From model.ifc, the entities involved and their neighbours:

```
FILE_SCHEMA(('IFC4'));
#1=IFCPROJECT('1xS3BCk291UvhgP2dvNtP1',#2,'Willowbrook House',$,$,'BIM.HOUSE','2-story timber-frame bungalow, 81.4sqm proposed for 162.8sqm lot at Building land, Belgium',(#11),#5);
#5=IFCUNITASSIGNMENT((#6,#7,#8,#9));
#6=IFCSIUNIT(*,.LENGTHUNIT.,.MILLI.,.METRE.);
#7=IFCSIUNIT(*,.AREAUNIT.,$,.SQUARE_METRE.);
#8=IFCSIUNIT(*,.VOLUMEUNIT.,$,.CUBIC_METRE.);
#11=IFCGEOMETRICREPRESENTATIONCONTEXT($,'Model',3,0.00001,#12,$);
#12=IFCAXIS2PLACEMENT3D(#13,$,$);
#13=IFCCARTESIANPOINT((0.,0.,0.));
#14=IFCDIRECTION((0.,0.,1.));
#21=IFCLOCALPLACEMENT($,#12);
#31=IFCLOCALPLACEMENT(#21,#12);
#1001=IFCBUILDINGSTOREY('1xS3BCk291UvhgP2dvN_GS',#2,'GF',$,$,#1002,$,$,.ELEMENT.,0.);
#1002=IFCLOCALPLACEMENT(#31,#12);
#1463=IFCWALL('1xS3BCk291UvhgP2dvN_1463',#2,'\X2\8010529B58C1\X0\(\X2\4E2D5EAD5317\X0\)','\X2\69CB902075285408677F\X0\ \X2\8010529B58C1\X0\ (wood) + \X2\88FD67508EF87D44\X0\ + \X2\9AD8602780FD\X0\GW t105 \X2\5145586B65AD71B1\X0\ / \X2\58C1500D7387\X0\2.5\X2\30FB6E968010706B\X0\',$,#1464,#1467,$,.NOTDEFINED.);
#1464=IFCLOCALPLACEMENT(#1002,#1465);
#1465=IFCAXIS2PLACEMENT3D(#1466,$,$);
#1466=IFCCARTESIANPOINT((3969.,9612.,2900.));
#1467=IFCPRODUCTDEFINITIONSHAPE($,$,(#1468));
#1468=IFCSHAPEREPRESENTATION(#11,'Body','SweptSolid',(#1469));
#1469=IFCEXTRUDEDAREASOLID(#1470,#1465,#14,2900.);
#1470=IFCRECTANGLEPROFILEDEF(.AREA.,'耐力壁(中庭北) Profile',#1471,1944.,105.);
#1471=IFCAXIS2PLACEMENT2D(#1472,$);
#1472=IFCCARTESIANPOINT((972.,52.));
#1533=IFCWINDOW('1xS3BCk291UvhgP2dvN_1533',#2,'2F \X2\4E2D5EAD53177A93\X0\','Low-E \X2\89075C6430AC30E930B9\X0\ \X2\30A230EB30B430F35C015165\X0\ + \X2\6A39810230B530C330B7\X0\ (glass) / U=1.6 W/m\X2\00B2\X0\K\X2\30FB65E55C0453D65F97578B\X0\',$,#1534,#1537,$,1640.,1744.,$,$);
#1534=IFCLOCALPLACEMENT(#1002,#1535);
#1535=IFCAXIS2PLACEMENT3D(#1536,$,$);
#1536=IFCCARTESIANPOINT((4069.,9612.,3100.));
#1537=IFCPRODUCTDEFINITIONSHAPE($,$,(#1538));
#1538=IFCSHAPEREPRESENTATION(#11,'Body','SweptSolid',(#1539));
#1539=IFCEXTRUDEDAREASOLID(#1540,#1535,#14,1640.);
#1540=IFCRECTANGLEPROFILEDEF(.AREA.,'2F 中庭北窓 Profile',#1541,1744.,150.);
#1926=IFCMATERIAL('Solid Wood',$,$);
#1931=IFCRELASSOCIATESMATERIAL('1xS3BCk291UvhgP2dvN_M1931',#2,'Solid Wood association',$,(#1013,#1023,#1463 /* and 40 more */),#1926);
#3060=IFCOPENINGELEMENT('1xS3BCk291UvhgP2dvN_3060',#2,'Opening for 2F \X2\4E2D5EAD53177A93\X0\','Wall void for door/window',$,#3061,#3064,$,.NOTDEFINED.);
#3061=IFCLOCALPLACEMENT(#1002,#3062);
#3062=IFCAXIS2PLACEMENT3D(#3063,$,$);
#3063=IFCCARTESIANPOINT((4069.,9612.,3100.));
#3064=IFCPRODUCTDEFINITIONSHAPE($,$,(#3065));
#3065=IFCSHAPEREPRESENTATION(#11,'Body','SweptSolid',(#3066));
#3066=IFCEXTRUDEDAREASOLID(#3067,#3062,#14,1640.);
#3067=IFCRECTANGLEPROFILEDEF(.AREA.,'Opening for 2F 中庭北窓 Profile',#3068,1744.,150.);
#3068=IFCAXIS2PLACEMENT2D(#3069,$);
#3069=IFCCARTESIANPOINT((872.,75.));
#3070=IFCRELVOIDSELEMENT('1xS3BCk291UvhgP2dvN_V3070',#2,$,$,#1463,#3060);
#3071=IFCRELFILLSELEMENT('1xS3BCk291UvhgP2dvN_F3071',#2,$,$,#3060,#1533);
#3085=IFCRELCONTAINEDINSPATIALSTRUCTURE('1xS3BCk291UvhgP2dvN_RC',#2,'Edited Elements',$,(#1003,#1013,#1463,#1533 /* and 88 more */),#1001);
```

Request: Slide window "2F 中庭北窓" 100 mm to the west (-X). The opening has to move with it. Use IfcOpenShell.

```python
import ifcopenshell
import ifcopenshell.api.geometry
import ifcopenshell.util.placement
import ifcopenshell.util.unit

model = ifcopenshell.open("model.ifc")
unit_scale = ifcopenshell.util.unit.calculate_unit_scale(model)

window = model.by_guid("1xS3BCk291UvhgP2dvN_1533")
opening = window.FillsVoids[0].RelatingOpeningElement
wall = opening.VoidsElements[0].RelatingBuildingElement

wall_matrix = ifcopenshell.util.placement.get_local_placement(wall.ObjectPlacement)
shift = wall_matrix[:3, 0] * -0.1 / unit_scale
before = ifcopenshell.util.placement.get_local_placement(window.ObjectPlacement)[:3, 3].copy()

# The window is not placed relative to its opening, so move both.
for product in (opening, window):
    matrix = ifcopenshell.util.placement.get_local_placement(product.ObjectPlacement)
    matrix[:3, 3] += shift
    ifcopenshell.api.geometry.edit_object_placement(model, product=product, matrix=matrix, is_si=False)

after = ifcopenshell.util.placement.get_local_placement(window.ObjectPlacement)[:3, 3]
print("window moved by", (after - before).round(3) + 0.0)

model.write("model-out.ifc")
```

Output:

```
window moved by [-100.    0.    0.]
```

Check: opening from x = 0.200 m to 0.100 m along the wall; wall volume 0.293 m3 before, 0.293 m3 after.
